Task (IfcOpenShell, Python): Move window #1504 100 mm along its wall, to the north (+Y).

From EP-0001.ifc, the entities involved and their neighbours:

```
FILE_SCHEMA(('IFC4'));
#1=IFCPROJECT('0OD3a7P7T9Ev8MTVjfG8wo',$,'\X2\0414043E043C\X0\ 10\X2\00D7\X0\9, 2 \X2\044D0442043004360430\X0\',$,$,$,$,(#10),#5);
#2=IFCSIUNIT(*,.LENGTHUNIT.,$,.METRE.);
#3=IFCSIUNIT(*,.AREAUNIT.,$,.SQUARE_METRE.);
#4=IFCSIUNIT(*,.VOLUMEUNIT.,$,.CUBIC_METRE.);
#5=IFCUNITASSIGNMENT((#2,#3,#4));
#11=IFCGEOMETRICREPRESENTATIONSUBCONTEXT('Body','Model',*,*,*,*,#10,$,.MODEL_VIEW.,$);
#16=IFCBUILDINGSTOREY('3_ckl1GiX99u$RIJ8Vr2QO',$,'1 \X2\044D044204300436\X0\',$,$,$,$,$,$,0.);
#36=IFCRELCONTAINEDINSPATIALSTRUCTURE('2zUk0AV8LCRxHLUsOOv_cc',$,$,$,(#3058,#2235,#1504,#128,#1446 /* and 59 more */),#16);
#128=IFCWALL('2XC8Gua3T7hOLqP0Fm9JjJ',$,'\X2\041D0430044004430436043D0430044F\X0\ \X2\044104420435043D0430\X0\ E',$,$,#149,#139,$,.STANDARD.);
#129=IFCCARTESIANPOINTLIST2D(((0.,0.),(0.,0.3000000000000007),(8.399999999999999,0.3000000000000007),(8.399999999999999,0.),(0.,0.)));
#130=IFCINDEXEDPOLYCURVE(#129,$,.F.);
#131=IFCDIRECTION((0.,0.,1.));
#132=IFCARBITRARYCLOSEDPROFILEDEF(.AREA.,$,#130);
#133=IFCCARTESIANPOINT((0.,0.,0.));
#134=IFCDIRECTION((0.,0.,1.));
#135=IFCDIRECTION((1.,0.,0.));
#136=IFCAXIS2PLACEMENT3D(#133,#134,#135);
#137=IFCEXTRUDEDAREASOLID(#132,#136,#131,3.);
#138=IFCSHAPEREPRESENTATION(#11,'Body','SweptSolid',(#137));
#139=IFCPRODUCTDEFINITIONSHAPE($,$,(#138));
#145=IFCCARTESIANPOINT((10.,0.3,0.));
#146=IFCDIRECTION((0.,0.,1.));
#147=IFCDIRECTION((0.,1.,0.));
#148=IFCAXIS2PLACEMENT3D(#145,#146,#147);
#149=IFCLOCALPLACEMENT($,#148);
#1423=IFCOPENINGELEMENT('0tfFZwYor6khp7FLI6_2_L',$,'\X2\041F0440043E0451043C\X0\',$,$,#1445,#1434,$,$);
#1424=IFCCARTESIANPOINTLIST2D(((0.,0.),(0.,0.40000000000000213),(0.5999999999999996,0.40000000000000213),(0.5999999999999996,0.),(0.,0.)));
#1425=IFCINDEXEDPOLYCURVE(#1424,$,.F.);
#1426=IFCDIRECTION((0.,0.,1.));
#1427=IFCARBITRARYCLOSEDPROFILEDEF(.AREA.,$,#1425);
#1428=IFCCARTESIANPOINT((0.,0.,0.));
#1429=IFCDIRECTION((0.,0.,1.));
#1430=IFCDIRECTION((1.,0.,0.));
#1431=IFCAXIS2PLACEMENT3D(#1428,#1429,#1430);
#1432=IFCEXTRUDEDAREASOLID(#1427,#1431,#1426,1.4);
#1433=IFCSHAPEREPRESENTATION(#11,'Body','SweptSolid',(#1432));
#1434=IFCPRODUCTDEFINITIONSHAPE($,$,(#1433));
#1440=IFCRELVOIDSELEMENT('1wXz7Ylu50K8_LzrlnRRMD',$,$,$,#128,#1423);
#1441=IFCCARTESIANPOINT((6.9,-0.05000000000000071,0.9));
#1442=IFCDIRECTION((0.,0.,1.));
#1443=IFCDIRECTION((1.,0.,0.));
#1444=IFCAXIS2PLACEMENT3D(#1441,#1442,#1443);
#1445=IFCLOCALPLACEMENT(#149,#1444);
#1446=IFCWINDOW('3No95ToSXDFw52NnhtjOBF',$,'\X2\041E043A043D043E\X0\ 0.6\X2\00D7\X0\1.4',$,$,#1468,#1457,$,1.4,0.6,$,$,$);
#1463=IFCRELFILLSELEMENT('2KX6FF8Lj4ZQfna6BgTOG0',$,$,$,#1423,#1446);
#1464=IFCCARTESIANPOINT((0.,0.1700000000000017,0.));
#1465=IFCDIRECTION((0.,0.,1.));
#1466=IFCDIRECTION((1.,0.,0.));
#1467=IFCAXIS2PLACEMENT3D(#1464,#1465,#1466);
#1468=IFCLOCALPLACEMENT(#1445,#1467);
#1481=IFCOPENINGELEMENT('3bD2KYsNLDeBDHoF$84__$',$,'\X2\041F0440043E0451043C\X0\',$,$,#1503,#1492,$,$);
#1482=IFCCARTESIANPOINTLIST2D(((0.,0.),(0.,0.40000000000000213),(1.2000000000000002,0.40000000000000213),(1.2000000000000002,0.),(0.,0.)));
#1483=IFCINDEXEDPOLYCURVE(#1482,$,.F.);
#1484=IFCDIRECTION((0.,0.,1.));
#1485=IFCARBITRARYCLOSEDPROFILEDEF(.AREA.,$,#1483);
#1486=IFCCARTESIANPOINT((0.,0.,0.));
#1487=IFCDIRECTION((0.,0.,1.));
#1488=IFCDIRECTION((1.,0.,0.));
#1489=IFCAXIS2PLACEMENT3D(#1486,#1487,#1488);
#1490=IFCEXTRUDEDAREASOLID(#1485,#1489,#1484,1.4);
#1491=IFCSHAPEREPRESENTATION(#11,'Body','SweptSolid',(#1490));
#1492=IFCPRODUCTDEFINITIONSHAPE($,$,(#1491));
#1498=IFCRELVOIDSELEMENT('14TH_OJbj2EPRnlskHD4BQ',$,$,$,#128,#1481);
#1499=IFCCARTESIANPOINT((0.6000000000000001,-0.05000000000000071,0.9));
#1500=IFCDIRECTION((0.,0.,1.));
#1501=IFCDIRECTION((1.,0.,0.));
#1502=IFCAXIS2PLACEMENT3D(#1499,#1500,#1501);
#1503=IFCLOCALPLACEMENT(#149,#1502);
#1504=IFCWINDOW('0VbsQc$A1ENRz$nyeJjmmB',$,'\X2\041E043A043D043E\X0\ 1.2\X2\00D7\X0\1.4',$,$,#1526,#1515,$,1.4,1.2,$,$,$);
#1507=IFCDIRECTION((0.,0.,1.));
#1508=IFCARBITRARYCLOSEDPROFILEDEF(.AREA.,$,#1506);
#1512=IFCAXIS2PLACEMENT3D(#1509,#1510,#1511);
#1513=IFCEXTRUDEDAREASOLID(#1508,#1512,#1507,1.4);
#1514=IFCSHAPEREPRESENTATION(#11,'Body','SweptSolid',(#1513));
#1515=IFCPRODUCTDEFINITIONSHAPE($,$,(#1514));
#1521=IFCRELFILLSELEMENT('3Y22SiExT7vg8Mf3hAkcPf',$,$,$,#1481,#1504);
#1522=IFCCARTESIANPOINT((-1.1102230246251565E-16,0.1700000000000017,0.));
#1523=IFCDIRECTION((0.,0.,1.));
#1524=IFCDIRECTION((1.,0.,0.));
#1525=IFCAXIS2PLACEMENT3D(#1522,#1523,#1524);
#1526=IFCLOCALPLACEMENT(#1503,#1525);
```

```python
import ifcopenshell
import ifcopenshell.api.geometry
import ifcopenshell.util.placement
import ifcopenshell.util.unit

model = ifcopenshell.open("EP-0001.ifc")
unit_scale = ifcopenshell.util.unit.calculate_unit_scale(model)

window = model.by_id(1504)
opening = window.FillsVoids[0].RelatingOpeningElement
wall = opening.VoidsElements[0].RelatingBuildingElement

wall_matrix = ifcopenshell.util.placement.get_local_placement(wall.ObjectPlacement)
shift = wall_matrix[:3, 0] * 0.1 / unit_scale
before = ifcopenshell.util.placement.get_local_placement(window.ObjectPlacement)[:3, 3].copy()

# The window is placed relative to its opening, so it follows when the opening moves.
matrix = ifcopenshell.util.placement.get_local_placement(opening.ObjectPlacement)
matrix[:3, 3] += shift
ifcopenshell.api.geometry.edit_object_placement(
    model, product=opening, matrix=matrix, is_si=False, should_transform_children=True
)

after = ifcopenshell.util.placement.get_local_placement(window.ObjectPlacement)[:3, 3]
print("window moved by", (after - before).round(3) + 0.0)

model.write("EP-0001_edited.ifc")
```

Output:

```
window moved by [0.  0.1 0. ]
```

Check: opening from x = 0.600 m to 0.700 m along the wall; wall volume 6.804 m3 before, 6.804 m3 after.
